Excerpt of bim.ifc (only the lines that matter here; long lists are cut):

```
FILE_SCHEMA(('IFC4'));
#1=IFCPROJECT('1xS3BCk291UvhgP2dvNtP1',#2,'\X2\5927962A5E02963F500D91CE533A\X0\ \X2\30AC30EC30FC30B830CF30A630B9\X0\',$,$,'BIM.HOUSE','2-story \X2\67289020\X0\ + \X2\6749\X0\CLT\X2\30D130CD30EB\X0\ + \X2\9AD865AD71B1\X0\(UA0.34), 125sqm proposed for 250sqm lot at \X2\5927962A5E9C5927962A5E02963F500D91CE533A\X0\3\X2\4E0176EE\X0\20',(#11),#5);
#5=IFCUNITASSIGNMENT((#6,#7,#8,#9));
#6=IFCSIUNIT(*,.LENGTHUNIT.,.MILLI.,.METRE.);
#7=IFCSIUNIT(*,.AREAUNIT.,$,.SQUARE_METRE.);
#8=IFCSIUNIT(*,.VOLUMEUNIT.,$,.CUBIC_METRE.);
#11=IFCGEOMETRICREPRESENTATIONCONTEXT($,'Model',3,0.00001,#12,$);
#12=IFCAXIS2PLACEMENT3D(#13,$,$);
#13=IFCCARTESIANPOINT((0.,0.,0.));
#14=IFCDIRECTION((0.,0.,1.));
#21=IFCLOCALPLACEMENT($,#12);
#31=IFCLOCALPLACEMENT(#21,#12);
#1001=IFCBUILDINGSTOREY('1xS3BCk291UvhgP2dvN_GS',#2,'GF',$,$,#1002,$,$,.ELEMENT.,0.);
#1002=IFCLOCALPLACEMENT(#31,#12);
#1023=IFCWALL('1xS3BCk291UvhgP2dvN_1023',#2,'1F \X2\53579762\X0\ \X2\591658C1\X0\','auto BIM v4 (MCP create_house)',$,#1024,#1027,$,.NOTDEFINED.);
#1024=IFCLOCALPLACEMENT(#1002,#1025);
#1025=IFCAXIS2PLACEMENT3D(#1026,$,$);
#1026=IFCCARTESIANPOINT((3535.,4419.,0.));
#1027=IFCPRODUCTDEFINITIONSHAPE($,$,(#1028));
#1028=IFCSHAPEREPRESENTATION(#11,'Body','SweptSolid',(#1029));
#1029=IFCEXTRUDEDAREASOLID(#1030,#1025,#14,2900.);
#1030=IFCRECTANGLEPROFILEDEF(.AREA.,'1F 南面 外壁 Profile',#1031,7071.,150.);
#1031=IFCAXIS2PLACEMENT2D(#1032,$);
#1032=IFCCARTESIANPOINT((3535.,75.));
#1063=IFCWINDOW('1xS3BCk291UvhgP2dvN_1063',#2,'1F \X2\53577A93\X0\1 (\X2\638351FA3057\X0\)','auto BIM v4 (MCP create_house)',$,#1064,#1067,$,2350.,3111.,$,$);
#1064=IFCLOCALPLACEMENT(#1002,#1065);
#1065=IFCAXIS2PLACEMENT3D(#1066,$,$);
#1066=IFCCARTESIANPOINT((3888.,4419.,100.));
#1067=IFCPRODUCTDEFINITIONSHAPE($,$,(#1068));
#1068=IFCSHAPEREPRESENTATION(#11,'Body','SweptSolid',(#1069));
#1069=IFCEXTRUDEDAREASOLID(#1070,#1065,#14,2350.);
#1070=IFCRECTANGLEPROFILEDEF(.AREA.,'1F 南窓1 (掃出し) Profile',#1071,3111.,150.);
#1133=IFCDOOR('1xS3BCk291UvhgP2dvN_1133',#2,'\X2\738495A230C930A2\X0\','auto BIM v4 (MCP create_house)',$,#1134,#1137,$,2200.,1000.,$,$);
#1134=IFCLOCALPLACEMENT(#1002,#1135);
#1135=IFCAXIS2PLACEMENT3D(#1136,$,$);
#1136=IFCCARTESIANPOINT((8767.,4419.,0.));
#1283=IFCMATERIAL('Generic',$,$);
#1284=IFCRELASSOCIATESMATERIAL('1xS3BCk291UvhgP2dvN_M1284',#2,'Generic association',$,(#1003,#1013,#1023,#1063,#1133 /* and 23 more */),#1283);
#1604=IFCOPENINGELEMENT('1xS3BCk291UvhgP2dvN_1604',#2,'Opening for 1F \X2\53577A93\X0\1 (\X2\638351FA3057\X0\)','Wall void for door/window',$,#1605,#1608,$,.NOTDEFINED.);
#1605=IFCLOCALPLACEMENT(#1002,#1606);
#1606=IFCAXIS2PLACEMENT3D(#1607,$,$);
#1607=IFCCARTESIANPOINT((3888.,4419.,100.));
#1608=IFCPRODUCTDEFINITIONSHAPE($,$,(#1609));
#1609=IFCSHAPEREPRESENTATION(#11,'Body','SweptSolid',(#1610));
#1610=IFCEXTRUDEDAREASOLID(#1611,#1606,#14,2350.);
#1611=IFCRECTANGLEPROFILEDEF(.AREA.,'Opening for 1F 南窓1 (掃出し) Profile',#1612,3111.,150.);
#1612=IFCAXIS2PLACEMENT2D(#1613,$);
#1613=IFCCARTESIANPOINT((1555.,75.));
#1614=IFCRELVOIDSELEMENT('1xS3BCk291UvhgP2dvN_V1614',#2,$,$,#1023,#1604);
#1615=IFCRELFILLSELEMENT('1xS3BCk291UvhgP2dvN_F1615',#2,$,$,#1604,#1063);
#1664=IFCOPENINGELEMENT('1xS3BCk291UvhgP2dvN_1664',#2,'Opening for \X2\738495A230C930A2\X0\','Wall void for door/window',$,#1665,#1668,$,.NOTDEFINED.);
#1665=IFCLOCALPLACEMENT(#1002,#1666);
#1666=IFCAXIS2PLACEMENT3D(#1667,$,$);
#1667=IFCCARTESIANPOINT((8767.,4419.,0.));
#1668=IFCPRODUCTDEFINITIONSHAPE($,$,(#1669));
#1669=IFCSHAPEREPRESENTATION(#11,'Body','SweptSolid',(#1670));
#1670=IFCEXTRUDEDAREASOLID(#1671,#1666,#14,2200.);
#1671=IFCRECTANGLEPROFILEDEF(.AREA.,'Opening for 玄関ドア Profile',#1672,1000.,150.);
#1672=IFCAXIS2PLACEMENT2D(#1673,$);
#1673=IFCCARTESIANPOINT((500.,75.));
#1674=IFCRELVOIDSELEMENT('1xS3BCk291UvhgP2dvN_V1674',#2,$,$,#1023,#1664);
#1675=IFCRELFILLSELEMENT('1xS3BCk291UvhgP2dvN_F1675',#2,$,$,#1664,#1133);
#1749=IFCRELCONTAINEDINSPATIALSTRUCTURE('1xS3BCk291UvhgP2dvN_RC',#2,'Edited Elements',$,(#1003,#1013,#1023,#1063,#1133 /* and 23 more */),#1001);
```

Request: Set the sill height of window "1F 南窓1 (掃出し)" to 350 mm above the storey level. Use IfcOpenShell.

```python
import numpy as np
import ifcopenshell
import ifcopenshell.api.geometry
import ifcopenshell.geom
import ifcopenshell.util.element
import ifcopenshell.util.placement
import ifcopenshell.util.shape
import ifcopenshell.util.unit

model = ifcopenshell.open("bim.ifc")
unit_scale = ifcopenshell.util.unit.calculate_unit_scale(model)

window = model.by_guid("1xS3BCk291UvhgP2dvN_1063")
opening = window.FillsVoids[0].RelatingOpeningElement
storey = ifcopenshell.util.element.get_container(window, ifc_class="IfcBuildingStorey")
level = ifcopenshell.util.placement.get_local_placement(storey.ObjectPlacement)[2, 3]

# The opening's origin need not be at the sill, so measure its lowest point.
shape = ifcopenshell.geom.create_shape(ifcopenshell.geom.settings(), opening)
bottom = ifcopenshell.util.shape.get_shape_bottom_elevation(shape, shape.geometry) / unit_scale
dz = level + 0.35 / unit_scale - bottom

shift = np.array([0.0, 0.0, dz])
# The window is not placed relative to its opening, so move both.
for product in (opening, window):
    matrix = ifcopenshell.util.placement.get_local_placement(product.ObjectPlacement)
    matrix[:3, 3] += shift
    ifcopenshell.api.geometry.edit_object_placement(model, product=product, matrix=matrix, is_si=False)

print(f"moved by {dz * unit_scale:+.3f} m")

model.write("bim_rev.ifc")
```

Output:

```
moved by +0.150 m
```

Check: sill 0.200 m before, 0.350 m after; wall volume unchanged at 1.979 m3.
